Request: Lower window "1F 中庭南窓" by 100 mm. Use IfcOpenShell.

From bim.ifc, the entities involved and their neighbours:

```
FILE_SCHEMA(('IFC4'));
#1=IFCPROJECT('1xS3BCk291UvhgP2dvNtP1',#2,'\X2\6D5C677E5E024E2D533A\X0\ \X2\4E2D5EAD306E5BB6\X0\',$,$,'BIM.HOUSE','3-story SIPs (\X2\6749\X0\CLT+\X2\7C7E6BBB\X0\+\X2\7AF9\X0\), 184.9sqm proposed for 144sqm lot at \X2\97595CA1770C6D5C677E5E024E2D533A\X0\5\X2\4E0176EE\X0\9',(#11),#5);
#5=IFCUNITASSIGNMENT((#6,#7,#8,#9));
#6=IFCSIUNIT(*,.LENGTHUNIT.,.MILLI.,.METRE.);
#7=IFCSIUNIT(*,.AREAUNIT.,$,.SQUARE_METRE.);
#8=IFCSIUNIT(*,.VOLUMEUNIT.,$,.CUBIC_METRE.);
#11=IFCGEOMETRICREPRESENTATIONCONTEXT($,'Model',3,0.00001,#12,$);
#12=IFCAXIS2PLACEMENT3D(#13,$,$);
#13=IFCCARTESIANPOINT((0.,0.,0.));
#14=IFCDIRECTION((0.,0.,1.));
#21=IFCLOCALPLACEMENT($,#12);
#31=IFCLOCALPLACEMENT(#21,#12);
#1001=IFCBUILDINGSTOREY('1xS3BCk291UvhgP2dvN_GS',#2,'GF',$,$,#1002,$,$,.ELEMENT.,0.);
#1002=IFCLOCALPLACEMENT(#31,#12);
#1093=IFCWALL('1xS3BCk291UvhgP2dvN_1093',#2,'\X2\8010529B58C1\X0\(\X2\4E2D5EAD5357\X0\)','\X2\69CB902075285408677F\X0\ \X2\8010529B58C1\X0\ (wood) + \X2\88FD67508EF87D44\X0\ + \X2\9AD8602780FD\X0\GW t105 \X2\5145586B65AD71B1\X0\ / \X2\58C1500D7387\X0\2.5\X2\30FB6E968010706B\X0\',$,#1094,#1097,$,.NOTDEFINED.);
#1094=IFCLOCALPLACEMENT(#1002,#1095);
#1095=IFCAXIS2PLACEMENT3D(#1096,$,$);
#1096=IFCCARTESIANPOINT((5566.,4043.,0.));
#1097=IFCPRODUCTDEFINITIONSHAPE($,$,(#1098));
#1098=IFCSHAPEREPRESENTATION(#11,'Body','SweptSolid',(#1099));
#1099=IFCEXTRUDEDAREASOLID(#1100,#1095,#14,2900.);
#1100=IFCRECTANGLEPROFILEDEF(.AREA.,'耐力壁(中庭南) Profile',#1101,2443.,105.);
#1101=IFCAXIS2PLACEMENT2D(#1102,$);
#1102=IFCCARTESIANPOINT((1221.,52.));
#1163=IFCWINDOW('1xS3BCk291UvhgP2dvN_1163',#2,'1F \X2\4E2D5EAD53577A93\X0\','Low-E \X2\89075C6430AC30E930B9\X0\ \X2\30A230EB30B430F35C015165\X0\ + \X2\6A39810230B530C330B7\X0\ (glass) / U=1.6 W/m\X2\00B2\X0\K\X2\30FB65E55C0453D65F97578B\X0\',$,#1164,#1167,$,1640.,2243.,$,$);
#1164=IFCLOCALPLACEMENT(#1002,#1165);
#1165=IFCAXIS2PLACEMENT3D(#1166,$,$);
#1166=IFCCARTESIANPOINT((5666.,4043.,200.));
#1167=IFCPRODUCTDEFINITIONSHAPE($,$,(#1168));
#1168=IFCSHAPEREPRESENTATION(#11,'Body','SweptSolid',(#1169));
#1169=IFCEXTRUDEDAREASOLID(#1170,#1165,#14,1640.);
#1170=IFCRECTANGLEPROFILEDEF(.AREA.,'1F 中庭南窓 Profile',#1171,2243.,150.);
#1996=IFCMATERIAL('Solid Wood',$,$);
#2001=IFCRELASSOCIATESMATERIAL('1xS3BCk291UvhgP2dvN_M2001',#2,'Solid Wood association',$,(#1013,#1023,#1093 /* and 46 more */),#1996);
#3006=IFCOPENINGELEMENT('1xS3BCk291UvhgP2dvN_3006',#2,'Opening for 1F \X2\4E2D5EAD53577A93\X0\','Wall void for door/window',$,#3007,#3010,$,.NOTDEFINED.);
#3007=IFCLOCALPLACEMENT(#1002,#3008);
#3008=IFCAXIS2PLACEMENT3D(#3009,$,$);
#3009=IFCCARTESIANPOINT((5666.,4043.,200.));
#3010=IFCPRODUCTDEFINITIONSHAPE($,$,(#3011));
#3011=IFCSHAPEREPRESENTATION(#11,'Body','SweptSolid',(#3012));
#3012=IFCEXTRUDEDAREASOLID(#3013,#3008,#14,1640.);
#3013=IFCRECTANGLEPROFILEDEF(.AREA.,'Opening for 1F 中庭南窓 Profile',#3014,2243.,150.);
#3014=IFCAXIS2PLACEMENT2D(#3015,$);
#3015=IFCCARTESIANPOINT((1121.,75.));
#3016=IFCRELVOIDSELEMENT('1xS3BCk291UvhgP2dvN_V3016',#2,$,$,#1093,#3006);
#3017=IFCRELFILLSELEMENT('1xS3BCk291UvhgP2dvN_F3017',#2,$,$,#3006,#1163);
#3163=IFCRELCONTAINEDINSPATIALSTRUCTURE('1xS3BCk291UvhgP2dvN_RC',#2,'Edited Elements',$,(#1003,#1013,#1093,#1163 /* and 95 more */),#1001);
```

```python
import numpy as np
import ifcopenshell
import ifcopenshell.api.geometry
import ifcopenshell.util.placement
import ifcopenshell.util.unit

model = ifcopenshell.open("bim.ifc")
unit_scale = ifcopenshell.util.unit.calculate_unit_scale(model)

window = model.by_guid("1xS3BCk291UvhgP2dvN_1163")
opening = window.FillsVoids[0].RelatingOpeningElement
dz = -100.0

shift = np.array([0.0, 0.0, dz])
# The window is not placed relative to its opening, so move both.
for product in (opening, window):
    matrix = ifcopenshell.util.placement.get_local_placement(product.ObjectPlacement)
    matrix[:3, 3] += shift
    ifcopenshell.api.geometry.edit_object_placement(model, product=product, matrix=matrix, is_si=False)

print(f"moved by {dz * unit_scale:+.3f} m")

model.write("bim-out.ifc")
```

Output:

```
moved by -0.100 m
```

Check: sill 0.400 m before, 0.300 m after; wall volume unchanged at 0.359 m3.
